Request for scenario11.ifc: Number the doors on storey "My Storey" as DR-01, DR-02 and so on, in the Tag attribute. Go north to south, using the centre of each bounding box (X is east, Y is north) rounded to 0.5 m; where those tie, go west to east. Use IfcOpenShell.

First a look at what the model holds.

```python
import ifcopenshell
import ifcopenshell.util.element
import ifcopenshell.util.placement

model = ifcopenshell.open("scenario11.ifc")
print(model.schema)
storey = next(s for s in model.by_type("IfcBuildingStorey") if s.Name == "My Storey")
doors = [e for e in ifcopenshell.util.element.get_decomposition(storey) if e.is_a("IfcDoor")]
for e in sorted(doors, key=lambda e: e.id()):
    origin = ifcopenshell.util.placement.get_local_placement(e.ObjectPlacement)[:3, 3]
    print(e.id(), e.Tag, e.Name, origin.round(2) + 0.0, sep=" | ")
```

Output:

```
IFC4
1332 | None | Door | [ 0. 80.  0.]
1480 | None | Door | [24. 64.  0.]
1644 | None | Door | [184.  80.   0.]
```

```python
import ifcopenshell
import ifcopenshell.geom
import ifcopenshell.util.element
import ifcopenshell.util.shape

model = ifcopenshell.open("scenario11.ifc")
settings = ifcopenshell.geom.settings()
settings.set("use-world-coords", True)


def centre(element):
    shape = ifcopenshell.geom.create_shape(settings, element)
    return ifcopenshell.util.shape.get_bbox_centroid(shape.geometry)


storey = next(s for s in model.by_type("IfcBuildingStorey") if s.Name == "My Storey")
doors = [e for e in ifcopenshell.util.element.get_decomposition(storey) if e.is_a("IfcDoor")]

# Insertion points can sit at a corner or the storey origin, so sort by the geometry (in metres).
centres = {e: centre(e) for e in doors}
doors.sort(key=lambda e: (-round(centres[e][1] / 0.5), centres[e][0]))

for i, e in enumerate(doors, start=1):
    number = f"DR-{i:02d}"
    e.Tag = number
    print(e.id(), number)

model.write("scenario11_v2.ifc")
```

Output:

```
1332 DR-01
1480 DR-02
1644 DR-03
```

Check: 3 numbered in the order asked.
